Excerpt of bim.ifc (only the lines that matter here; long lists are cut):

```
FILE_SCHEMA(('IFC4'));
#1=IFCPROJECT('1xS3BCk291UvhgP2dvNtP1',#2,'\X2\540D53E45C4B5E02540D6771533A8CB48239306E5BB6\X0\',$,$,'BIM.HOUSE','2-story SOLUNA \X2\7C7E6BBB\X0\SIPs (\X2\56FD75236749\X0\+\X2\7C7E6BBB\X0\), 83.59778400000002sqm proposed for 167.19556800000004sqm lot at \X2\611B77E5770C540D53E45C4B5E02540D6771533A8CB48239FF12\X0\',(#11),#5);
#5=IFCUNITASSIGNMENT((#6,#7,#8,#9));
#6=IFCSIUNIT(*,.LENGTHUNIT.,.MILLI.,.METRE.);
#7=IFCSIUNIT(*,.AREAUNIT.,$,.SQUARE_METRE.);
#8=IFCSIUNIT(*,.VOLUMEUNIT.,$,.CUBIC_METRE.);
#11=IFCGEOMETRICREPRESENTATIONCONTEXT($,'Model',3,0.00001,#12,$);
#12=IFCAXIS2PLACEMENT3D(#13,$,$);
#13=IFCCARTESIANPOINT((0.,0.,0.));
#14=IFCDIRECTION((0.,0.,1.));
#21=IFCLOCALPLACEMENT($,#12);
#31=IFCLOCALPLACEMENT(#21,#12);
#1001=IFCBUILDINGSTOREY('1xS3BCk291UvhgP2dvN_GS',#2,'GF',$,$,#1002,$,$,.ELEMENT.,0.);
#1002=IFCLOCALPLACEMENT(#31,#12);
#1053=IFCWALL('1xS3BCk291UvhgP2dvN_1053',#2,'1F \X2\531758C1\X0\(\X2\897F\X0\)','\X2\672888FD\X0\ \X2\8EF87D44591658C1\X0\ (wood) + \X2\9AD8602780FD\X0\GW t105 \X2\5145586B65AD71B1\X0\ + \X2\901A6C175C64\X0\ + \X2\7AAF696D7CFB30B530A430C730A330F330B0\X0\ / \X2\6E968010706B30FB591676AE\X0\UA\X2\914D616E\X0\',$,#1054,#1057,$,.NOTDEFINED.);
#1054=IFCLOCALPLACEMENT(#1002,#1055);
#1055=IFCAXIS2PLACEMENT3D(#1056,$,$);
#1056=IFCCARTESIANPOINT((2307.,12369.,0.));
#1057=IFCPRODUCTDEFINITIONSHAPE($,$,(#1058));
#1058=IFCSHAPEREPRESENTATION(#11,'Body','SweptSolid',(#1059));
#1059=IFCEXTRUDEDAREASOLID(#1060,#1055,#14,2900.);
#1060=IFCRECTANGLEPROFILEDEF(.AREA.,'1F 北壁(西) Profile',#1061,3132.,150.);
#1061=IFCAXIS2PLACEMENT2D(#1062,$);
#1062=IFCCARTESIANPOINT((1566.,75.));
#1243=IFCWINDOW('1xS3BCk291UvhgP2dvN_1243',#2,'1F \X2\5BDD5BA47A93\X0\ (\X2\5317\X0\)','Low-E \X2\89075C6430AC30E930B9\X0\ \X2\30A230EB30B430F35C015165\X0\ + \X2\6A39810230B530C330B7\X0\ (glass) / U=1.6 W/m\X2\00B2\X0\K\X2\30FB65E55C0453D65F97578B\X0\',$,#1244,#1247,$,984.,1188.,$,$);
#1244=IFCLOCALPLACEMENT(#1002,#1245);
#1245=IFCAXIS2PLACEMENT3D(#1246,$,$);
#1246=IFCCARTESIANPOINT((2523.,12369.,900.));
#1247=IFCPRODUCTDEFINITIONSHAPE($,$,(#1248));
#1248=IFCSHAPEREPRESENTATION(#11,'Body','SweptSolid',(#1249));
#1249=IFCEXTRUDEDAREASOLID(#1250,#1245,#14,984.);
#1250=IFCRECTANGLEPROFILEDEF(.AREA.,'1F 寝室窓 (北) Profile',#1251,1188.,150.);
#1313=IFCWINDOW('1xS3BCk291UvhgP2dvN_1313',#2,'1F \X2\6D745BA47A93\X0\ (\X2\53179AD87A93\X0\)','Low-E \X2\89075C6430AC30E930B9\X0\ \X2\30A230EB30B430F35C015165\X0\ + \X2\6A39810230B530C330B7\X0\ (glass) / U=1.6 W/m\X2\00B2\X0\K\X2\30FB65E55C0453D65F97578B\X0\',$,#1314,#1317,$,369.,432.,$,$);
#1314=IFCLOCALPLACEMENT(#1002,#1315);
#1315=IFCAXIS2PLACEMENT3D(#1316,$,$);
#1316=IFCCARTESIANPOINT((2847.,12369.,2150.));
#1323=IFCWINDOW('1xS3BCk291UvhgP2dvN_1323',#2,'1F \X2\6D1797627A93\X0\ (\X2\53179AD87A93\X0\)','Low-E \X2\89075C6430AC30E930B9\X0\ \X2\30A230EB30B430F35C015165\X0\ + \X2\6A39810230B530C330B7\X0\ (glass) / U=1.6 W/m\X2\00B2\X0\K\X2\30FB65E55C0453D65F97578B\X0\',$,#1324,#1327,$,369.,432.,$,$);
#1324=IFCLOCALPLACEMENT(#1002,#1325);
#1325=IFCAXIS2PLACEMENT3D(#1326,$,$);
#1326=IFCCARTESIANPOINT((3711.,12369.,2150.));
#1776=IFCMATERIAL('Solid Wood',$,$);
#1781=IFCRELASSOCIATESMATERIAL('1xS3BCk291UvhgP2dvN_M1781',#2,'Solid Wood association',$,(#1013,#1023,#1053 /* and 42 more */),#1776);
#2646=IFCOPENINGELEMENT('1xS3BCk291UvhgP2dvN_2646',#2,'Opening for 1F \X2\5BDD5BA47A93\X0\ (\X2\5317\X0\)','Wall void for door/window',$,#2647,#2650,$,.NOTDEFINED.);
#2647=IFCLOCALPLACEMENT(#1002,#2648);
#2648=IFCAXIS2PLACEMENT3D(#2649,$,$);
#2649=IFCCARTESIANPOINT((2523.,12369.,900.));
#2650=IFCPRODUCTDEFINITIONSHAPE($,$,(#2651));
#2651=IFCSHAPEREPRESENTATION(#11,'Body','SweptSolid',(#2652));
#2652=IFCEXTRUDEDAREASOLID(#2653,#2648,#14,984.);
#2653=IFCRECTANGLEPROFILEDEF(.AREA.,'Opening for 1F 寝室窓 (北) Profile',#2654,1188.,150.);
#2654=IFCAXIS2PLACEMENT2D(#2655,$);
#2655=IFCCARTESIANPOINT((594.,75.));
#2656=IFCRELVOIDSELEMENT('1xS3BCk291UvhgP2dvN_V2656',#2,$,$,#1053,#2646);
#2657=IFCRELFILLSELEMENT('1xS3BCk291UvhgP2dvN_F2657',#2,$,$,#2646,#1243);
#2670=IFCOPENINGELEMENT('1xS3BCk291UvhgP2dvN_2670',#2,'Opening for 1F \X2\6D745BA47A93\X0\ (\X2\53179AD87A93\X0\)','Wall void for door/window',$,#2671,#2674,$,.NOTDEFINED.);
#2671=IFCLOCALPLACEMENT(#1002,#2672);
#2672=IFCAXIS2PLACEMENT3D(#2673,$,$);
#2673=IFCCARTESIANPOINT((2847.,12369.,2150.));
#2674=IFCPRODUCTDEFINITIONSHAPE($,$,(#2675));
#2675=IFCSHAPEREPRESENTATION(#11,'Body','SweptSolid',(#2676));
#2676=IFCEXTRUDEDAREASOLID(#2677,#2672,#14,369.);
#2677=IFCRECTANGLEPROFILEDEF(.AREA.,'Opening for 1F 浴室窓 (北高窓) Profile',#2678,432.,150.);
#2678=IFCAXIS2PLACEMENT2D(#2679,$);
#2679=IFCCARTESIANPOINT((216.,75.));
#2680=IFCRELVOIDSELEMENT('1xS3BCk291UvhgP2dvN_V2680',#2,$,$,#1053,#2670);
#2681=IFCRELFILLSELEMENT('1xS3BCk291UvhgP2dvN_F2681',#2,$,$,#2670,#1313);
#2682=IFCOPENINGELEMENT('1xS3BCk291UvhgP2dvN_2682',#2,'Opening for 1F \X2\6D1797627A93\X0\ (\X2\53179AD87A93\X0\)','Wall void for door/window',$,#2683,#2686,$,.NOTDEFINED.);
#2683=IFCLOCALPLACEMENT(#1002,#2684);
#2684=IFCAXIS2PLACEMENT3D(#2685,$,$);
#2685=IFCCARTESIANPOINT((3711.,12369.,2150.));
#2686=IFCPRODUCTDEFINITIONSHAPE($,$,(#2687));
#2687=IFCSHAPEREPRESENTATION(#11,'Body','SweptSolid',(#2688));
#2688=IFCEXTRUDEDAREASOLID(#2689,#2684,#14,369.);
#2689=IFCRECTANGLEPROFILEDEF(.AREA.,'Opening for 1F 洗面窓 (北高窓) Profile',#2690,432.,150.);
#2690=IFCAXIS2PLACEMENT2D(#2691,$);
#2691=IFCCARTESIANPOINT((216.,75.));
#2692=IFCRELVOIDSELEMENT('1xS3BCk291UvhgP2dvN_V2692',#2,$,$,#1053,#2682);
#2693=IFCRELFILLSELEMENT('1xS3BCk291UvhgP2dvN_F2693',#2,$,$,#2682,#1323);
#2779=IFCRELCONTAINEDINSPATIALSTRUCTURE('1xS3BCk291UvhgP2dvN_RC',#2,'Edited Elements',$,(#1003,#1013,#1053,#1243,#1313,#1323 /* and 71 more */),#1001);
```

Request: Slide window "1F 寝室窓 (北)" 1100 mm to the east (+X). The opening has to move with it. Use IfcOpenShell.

```python
import ifcopenshell
import ifcopenshell.api.geometry
import ifcopenshell.util.placement
import ifcopenshell.util.unit

model = ifcopenshell.open("bim.ifc")
unit_scale = ifcopenshell.util.unit.calculate_unit_scale(model)

window = model.by_guid("1xS3BCk291UvhgP2dvN_1243")
opening = window.FillsVoids[0].RelatingOpeningElement
wall = opening.VoidsElements[0].RelatingBuildingElement

wall_matrix = ifcopenshell.util.placement.get_local_placement(wall.ObjectPlacement)
shift = wall_matrix[:3, 0] * 1.1 / unit_scale
before = ifcopenshell.util.placement.get_local_placement(window.ObjectPlacement)[:3, 3].copy()

# The window is not placed relative to its opening, so move both.
for product in (opening, window):
    matrix = ifcopenshell.util.placement.get_local_placement(product.ObjectPlacement)
    matrix[:3, 3] += shift
    ifcopenshell.api.geometry.edit_object_placement(model, product=product, matrix=matrix, is_si=False)

after = ifcopenshell.util.placement.get_local_placement(window.ObjectPlacement)[:3, 3]
print("window moved by", (after - before).round(3) + 0.0)

model.write("bim_updated.ifc")
```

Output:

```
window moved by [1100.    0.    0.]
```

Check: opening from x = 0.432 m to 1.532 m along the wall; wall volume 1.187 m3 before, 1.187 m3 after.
